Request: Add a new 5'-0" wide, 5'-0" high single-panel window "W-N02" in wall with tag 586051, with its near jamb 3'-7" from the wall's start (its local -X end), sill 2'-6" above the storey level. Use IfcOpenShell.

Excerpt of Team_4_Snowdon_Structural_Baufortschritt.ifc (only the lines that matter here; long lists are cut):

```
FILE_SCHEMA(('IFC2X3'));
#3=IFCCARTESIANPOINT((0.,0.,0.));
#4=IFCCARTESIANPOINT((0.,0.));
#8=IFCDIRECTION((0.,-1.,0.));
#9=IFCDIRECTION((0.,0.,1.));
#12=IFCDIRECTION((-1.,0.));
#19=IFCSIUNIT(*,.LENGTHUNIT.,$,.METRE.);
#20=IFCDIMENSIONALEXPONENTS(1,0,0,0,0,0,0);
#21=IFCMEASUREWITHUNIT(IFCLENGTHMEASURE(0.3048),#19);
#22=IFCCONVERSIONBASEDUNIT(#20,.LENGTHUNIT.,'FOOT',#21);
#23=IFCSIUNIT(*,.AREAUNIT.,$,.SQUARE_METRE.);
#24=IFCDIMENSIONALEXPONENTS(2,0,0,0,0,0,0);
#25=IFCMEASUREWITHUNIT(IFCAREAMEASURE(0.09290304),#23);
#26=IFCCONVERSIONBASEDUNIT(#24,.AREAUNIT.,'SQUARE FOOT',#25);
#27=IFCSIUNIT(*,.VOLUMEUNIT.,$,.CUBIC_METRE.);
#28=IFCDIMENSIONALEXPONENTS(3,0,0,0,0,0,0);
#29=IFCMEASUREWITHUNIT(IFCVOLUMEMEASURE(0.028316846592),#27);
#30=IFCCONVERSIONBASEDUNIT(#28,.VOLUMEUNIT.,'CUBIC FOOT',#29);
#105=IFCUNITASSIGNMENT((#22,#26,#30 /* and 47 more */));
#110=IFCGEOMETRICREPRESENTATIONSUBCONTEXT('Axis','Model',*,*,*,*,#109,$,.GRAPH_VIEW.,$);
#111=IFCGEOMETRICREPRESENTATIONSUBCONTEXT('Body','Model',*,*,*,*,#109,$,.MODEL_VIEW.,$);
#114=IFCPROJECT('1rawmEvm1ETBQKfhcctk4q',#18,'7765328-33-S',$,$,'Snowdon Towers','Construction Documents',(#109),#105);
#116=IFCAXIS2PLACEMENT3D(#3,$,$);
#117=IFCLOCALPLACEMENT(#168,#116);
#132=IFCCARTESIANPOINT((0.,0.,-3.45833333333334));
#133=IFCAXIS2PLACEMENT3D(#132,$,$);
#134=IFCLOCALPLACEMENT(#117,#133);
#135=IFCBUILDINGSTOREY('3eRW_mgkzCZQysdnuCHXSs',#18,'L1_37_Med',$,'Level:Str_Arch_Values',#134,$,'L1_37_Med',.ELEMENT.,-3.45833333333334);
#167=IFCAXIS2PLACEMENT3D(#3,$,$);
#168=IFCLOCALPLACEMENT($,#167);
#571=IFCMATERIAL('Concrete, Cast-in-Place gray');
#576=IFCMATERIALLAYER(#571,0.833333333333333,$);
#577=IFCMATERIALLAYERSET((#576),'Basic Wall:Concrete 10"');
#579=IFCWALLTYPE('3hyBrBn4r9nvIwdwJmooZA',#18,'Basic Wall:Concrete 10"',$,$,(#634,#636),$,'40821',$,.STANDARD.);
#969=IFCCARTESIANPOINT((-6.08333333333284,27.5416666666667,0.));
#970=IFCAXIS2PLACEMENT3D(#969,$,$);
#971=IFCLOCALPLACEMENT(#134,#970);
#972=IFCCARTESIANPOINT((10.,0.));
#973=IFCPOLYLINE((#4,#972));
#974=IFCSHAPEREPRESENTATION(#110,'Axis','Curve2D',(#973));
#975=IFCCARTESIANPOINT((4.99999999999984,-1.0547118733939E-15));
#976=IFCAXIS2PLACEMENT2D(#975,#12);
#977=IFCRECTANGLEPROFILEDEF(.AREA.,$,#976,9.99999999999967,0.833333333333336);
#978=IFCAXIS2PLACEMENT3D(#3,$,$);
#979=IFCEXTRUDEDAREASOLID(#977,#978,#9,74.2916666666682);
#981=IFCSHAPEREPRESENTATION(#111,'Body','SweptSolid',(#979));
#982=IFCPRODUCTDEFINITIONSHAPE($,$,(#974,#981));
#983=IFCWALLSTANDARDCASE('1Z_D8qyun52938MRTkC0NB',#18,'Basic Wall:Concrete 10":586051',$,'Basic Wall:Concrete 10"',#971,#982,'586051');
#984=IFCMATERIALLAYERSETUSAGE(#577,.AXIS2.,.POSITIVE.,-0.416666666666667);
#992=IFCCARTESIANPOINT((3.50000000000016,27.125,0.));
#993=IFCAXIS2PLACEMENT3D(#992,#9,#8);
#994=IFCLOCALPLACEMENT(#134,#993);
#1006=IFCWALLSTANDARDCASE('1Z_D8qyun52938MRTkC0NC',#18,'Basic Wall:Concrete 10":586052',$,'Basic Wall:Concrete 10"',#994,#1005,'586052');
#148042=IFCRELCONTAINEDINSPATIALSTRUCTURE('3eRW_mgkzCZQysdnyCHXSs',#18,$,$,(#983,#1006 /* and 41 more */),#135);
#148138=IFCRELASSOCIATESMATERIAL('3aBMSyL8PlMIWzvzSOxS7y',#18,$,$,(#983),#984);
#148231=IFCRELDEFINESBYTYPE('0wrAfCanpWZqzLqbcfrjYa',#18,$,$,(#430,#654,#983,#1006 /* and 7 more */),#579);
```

```python
import numpy as np
import ifcopenshell
import ifcopenshell.api.feature
import ifcopenshell.api.geometry
import ifcopenshell.api.root
import ifcopenshell.api.spatial
import ifcopenshell.api.type
import ifcopenshell.geom
import ifcopenshell.util.element
import ifcopenshell.util.placement
import ifcopenshell.util.representation
import ifcopenshell.util.shape
import ifcopenshell.util.unit

model = ifcopenshell.open("Team_4_Snowdon_Structural_Baufortschritt.ifc")
unit_scale = ifcopenshell.util.unit.calculate_unit_scale(model)
settings = ifcopenshell.geom.settings()


def volume(element):
    """Net volume in cubic metres, openings subtracted."""
    shape = ifcopenshell.geom.create_shape(settings, element)
    return ifcopenshell.util.shape.get_volume(shape.geometry)


wall = model.by_guid("1Z_D8qyun52938MRTkC0NB")
storey = ifcopenshell.util.element.get_container(wall, ifc_class="IfcBuildingStorey")
context = ifcopenshell.util.representation.get_context(model, "Model", "Body", "MODEL_VIEW")
before = volume(wall)

width, height, from_end, sill = 1.524, 1.524, 1.0922, 0.762  # metres

# The wall runs along its own X axis, and the end named is its -X end.
wall_shape = ifcopenshell.geom.create_shape(settings, wall)
x, y, z = ifcopenshell.util.shape.get_vertices(wall_shape.geometry).T
start = x.min() + from_end
face, thickness = float(y.min()), float(y.max() - y.min())
wall_matrix = ifcopenshell.util.placement.get_local_placement(wall.ObjectPlacement)
level = ifcopenshell.util.placement.get_local_placement(storey.ObjectPlacement)[2, 3]


def in_wall(x, y):
    """Placement at x, y metres in the wall's axes, at sill height."""
    matrix = wall_matrix.copy()
    matrix[:, 3] = wall_matrix @ np.array([x / unit_scale, y / unit_scale, 0.0, 1.0])
    matrix[2, 3] = level + sill / unit_scale
    return matrix


# Opening: a box that overshoots both wall faces by 50 mm.
opening = ifcopenshell.api.root.create_entity(model, ifc_class="IfcOpeningElement")
box = ifcopenshell.api.geometry.add_wall_representation(
    model, context=context, length=width, height=height, thickness=thickness + 0.1
)
ifcopenshell.api.geometry.assign_representation(model, product=opening, representation=box)
ifcopenshell.api.geometry.edit_object_placement(model, product=opening, matrix=in_wall(start, face - 0.05), is_si=False)
ifcopenshell.api.feature.add_feature(model, feature=opening, element=wall)

window = ifcopenshell.api.root.create_entity(model, ifc_class="IfcWindow", name="W-N02")
window.OverallWidth, window.OverallHeight = width / unit_scale, height / unit_scale
body = ifcopenshell.api.geometry.add_window_representation(
    model,
    context=context,
    overall_width=window.OverallWidth,
    overall_height=window.OverallHeight,
    partition_type="SINGLE_PANEL",
)
ifcopenshell.api.geometry.assign_representation(model, product=window, representation=body)
ifcopenshell.api.spatial.assign_container(model, products=[window], relating_structure=storey)
fills = ifcopenshell.api.feature.add_filling(model, opening=opening, element=window)
fills.OwnerHistory = window.OwnerHistory  # required in IFC2X3

# IFC2X3 keeps the operation on the window style.
style = ifcopenshell.api.root.create_entity(model, ifc_class="IfcWindowStyle", name="W-N02")
style.OperationType, style.ConstructionType = "SINGLE_PANEL", "NOTDEFINED"
style.ParameterTakesPrecedence = style.Sizeable = False
ifcopenshell.api.type.assign_type(model, related_objects=[window], relating_type=style)

# Centre the window in the wall's thickness.
ifcopenshell.api.geometry.edit_object_placement(model, product=window, matrix=in_wall(start, face), is_si=False)
window_shape = ifcopenshell.geom.create_shape(settings, window)
depth = ifcopenshell.util.shape.get_vertices(window_shape.geometry)[:, 1]
offset = face + thickness / 2 - (depth.min() + depth.max()) / 2
ifcopenshell.api.geometry.edit_object_placement(model, product=window, matrix=in_wall(start, offset), is_si=False)

after = volume(wall)

print(f"wall volume {before:.3f} -> {after:.3f} m3")

model.write("Team_4_Snowdon_Structural_Baufortschritt_edited.ifc")
```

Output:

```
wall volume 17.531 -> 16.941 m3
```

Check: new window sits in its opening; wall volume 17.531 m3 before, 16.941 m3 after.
